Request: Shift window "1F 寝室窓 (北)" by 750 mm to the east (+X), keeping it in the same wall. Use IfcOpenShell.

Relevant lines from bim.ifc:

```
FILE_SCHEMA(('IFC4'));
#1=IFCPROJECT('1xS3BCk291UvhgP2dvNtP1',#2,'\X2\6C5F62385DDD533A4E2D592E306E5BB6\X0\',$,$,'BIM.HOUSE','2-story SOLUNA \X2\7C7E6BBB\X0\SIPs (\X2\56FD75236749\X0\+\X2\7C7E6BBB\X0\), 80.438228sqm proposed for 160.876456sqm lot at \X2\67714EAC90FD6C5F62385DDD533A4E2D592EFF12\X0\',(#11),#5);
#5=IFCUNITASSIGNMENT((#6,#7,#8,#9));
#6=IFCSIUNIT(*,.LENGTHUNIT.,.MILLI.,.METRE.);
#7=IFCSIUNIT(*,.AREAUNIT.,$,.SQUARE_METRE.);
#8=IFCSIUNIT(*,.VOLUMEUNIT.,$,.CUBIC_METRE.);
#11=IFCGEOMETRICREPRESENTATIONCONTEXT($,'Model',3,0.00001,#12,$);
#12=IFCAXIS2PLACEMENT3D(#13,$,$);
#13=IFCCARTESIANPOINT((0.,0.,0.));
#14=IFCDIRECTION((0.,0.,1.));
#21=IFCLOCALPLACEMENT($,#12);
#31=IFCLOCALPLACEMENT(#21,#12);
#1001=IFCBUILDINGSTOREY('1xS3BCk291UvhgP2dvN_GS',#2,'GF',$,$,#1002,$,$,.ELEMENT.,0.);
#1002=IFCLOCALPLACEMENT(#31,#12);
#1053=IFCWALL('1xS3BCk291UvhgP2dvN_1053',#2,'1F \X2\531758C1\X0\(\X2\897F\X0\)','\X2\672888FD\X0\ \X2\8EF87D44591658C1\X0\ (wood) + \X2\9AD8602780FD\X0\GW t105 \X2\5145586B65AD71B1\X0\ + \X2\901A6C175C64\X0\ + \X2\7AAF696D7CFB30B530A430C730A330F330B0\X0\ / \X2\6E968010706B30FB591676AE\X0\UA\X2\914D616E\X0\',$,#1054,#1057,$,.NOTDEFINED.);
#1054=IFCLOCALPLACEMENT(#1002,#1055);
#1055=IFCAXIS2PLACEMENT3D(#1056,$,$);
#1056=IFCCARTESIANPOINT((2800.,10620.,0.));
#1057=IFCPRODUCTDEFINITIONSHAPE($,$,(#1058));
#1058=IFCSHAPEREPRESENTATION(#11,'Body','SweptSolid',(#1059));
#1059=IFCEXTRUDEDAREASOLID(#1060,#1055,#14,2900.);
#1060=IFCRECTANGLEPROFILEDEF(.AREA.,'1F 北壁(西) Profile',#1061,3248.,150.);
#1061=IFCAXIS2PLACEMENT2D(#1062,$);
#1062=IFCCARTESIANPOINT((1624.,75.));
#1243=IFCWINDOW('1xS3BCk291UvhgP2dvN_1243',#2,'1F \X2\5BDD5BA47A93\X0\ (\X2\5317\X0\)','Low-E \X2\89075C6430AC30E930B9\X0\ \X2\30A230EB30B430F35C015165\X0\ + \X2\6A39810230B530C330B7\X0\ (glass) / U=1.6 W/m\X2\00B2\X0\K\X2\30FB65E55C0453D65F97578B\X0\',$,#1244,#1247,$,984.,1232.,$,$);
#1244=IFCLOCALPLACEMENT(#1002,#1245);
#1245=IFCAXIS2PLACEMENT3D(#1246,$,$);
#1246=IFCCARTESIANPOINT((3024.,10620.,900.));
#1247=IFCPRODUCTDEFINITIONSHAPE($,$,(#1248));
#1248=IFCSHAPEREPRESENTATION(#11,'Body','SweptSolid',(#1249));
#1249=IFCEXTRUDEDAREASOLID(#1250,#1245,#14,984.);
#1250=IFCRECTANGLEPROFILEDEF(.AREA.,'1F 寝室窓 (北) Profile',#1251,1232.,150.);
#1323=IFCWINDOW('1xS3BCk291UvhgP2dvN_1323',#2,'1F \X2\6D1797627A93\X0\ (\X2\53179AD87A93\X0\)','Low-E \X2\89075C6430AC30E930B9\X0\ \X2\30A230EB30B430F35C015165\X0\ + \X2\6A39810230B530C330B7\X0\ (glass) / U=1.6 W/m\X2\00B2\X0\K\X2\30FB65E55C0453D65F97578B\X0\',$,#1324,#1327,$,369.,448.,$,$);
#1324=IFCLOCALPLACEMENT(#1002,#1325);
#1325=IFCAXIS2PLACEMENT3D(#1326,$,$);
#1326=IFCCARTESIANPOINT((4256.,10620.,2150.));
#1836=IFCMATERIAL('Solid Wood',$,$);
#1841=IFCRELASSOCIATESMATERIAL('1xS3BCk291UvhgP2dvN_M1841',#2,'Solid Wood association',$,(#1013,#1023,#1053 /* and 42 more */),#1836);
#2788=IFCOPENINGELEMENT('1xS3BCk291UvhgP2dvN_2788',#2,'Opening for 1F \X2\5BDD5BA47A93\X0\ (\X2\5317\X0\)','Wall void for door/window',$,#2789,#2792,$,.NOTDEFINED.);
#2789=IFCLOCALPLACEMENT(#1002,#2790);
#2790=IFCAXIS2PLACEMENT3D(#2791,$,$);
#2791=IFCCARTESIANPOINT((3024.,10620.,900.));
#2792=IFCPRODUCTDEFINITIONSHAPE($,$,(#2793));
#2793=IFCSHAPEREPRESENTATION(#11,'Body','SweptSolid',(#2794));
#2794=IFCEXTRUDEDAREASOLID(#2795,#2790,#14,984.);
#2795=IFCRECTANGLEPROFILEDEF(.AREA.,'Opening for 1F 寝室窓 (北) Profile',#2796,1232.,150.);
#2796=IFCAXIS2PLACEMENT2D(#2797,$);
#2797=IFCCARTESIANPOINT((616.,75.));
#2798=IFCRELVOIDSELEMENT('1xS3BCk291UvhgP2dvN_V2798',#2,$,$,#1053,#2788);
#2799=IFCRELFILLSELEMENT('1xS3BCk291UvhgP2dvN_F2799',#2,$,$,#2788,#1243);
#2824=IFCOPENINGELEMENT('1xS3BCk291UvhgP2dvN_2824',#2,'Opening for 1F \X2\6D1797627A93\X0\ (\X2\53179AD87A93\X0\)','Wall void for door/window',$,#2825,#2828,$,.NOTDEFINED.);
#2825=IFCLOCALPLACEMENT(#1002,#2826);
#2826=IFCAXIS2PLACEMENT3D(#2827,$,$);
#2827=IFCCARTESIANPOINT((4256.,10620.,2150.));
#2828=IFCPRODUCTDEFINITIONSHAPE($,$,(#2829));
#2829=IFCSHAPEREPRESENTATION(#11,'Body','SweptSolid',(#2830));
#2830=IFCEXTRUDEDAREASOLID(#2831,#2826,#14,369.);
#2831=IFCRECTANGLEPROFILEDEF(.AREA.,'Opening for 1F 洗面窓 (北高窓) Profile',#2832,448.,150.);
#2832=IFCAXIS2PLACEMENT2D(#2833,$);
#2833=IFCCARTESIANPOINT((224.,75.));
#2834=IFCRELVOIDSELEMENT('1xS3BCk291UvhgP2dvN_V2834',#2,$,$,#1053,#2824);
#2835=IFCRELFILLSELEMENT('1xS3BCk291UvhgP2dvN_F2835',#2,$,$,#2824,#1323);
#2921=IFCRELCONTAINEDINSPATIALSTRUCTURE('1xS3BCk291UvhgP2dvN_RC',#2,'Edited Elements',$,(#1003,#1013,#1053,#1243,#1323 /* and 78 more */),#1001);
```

```python
import ifcopenshell
import ifcopenshell.api.geometry
import ifcopenshell.util.placement
import ifcopenshell.util.unit

model = ifcopenshell.open("bim.ifc")
unit_scale = ifcopenshell.util.unit.calculate_unit_scale(model)

window = model.by_guid("1xS3BCk291UvhgP2dvN_1243")
opening = window.FillsVoids[0].RelatingOpeningElement
wall = opening.VoidsElements[0].RelatingBuildingElement

wall_matrix = ifcopenshell.util.placement.get_local_placement(wall.ObjectPlacement)
shift = wall_matrix[:3, 0] * 0.75 / unit_scale
before = ifcopenshell.util.placement.get_local_placement(window.ObjectPlacement)[:3, 3].copy()

# The window is not placed relative to its opening, so move both.
for product in (opening, window):
    matrix = ifcopenshell.util.placement.get_local_placement(product.ObjectPlacement)
    matrix[:3, 3] += shift
    ifcopenshell.api.geometry.edit_object_placement(model, product=product, matrix=matrix, is_si=False)

after = ifcopenshell.util.placement.get_local_placement(window.ObjectPlacement)[:3, 3]
print("window moved by", (after - before).round(3) + 0.0)

model.write("bim_edited.ifc")
```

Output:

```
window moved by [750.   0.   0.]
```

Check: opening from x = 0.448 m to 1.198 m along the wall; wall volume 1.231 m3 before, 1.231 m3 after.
